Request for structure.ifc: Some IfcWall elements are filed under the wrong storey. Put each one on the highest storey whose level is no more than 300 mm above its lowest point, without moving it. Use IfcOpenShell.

First a look at what the model holds.

```python
import ifcopenshell
import ifcopenshell.util.element
import ifcopenshell.util.placement

model = ifcopenshell.open("structure.ifc")
print(model.schema)
for storey in model.by_type("IfcBuildingStorey"):
    level = ifcopenshell.util.placement.get_storey_elevation(storey)
    count = sum(e.is_a("IfcWall") for e in ifcopenshell.util.element.get_contained(storey))
    print(storey.id(), storey.Name, round(level, 3), count, sep=" | ")
```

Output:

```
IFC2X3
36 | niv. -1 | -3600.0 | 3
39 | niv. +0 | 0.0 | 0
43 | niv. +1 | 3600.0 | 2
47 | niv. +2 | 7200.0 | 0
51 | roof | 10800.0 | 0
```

```python
import ifcopenshell
import ifcopenshell.api.spatial
import ifcopenshell.geom
import ifcopenshell.util.element
import ifcopenshell.util.placement
import ifcopenshell.util.shape
import ifcopenshell.util.unit

model = ifcopenshell.open("structure.ifc")
unit_scale = ifcopenshell.util.unit.calculate_unit_scale(model)
settings = ifcopenshell.geom.settings()

levels = sorted(
    ((ifcopenshell.util.placement.get_storey_elevation(s) * unit_scale, s) for s in model.by_type("IfcBuildingStorey")),
    key=lambda pair: pair[0],
)

for e in model.by_type("IfcWall"):
    current = e.ContainedInStructure[0].RelatingStructure if e.ContainedInStructure else None
    if current is None or not current.is_a("IfcBuildingStorey"):
        continue
    shape = ifcopenshell.geom.create_shape(settings, e)
    bottom = ifcopenshell.util.shape.get_shape_bottom_elevation(shape, shape.geometry)
    below = [s for level, s in levels if level <= bottom + 0.3]
    storey = below[-1] if below else levels[0][1]
    if storey != current:
        # assign_container keeps the world position.
        ifcopenshell.api.spatial.assign_container(model, products=[e], relating_structure=storey)
        print(e.id(), current.Name, "->", storey.Name)

model.write("structure_v2.ifc")
```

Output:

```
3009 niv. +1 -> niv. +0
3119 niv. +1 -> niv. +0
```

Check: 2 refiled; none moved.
